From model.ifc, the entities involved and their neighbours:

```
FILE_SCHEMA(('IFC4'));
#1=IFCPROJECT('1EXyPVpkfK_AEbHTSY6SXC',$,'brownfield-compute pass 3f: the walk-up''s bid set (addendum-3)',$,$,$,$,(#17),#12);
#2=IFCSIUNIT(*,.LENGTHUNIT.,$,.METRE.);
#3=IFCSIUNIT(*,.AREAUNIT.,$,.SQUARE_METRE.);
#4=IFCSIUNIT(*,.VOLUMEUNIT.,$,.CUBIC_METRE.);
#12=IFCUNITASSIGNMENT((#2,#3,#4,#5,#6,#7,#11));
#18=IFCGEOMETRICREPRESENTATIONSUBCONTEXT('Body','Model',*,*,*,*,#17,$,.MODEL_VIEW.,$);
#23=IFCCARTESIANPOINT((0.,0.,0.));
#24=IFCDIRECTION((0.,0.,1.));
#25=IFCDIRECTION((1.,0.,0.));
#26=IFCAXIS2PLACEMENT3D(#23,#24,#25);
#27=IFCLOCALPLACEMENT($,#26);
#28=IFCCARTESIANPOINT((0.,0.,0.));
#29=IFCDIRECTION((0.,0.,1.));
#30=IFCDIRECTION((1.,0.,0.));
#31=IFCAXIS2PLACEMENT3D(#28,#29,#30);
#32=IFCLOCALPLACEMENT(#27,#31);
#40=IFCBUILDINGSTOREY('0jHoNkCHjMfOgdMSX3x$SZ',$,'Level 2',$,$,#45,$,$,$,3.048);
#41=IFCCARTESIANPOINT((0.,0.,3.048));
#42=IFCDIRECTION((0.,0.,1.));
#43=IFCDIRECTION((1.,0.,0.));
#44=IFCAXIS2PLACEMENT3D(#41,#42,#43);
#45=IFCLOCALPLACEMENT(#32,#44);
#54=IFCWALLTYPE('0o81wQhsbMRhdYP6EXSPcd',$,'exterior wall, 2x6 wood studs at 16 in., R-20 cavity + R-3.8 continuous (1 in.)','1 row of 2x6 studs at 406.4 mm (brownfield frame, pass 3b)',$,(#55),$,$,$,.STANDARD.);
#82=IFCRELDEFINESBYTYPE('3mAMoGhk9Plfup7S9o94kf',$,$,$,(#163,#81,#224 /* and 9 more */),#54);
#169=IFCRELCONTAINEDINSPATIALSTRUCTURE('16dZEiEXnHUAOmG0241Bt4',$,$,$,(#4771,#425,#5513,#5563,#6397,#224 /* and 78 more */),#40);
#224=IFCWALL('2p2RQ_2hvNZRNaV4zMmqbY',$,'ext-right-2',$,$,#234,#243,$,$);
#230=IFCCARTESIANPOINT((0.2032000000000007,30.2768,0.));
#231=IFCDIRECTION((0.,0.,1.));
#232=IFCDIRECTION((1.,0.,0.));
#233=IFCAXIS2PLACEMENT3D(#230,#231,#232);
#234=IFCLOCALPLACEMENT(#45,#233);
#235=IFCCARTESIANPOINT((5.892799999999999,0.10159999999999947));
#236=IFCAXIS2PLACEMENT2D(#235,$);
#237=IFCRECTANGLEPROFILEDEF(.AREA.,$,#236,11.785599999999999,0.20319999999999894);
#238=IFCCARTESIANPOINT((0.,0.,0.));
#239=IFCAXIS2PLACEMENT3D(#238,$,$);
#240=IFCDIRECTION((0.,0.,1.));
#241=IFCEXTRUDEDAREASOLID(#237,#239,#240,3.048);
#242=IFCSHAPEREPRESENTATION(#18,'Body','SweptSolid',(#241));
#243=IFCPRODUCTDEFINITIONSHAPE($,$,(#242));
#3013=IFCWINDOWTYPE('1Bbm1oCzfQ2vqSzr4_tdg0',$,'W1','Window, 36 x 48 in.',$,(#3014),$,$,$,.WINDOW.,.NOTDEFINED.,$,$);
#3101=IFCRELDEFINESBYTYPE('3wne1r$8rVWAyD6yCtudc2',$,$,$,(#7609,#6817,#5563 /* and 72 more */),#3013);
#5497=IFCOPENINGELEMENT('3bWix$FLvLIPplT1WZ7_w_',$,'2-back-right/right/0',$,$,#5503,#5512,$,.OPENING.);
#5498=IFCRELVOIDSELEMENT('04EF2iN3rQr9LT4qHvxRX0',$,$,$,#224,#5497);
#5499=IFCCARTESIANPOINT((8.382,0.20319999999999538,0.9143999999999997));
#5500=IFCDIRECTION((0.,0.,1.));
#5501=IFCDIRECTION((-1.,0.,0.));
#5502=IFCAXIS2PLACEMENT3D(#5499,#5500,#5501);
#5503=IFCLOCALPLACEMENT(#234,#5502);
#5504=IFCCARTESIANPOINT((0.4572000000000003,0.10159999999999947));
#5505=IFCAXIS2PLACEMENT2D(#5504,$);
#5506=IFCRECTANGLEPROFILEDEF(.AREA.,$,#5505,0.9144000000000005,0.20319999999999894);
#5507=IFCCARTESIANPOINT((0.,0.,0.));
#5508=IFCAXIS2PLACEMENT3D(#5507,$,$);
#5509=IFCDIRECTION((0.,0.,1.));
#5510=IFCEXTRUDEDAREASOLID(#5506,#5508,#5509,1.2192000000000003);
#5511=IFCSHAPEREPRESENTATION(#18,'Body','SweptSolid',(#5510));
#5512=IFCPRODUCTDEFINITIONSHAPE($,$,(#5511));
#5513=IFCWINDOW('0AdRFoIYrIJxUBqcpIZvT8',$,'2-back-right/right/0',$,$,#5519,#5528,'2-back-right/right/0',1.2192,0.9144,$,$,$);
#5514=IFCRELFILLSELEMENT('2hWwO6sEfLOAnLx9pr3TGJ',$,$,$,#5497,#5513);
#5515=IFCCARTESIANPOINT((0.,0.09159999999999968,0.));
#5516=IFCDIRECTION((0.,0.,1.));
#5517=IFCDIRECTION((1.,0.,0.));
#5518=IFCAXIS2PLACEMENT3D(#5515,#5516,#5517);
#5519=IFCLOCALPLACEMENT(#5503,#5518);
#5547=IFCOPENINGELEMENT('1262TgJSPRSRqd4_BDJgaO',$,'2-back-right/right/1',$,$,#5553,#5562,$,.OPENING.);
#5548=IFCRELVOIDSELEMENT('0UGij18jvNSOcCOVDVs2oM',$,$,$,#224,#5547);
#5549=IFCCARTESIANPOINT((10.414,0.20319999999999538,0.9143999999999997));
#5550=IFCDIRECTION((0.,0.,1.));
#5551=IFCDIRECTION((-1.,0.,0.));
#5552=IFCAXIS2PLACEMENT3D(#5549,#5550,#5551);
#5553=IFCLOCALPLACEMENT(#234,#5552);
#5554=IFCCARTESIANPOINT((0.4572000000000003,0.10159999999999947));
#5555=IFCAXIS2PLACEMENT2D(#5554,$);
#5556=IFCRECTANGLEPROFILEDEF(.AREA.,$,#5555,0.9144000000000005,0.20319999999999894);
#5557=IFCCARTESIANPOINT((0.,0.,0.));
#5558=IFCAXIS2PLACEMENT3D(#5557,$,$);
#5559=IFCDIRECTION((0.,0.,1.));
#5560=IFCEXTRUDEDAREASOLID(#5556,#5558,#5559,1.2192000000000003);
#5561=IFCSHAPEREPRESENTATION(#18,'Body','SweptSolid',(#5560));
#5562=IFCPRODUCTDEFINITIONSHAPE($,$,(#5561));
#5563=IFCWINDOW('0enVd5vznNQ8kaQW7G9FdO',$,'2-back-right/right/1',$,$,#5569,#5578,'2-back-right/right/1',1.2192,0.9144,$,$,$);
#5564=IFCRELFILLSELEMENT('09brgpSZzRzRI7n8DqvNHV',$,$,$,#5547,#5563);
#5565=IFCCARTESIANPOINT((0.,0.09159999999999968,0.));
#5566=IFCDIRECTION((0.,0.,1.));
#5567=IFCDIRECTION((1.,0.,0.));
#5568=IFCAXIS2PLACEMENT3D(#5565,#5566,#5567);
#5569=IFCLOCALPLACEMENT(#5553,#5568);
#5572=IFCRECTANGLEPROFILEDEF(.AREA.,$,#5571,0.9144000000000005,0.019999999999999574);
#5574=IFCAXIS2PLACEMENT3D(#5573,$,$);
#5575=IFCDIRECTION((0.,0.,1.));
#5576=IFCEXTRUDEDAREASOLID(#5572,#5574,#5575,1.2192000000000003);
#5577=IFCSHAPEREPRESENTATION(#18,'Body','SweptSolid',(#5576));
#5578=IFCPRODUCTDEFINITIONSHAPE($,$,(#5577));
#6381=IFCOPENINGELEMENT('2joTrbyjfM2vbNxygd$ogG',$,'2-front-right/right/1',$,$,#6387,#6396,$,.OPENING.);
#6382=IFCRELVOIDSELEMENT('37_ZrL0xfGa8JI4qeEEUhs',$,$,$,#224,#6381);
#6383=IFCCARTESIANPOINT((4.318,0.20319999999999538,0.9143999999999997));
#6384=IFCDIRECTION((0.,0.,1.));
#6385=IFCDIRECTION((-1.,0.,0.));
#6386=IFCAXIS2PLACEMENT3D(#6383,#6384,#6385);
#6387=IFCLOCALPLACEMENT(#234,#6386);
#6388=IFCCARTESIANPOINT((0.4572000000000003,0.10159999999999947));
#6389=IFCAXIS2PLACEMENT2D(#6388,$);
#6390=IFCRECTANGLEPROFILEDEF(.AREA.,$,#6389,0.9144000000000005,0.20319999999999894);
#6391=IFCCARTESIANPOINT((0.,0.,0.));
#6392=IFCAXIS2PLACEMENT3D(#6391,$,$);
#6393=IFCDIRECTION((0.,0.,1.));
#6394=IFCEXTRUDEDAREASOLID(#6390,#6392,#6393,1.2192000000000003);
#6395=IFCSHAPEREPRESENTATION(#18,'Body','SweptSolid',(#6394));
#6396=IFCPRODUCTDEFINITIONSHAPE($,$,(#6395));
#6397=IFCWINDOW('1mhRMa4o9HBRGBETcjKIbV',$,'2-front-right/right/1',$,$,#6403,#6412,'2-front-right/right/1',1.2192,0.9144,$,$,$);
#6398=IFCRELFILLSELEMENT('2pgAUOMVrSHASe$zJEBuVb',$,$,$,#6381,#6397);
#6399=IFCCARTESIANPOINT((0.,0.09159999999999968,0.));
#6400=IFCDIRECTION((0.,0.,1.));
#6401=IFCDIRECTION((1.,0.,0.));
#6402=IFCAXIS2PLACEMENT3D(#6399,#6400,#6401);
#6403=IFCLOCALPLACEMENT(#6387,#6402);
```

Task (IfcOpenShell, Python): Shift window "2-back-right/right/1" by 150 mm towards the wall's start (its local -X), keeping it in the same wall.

```python
import ifcopenshell
import ifcopenshell.api.geometry
import ifcopenshell.util.placement

model = ifcopenshell.open("model.ifc")

window = model.by_guid("0enVd5vznNQ8kaQW7G9FdO")
opening = window.FillsVoids[0].RelatingOpeningElement
wall = opening.VoidsElements[0].RelatingBuildingElement

wall_matrix = ifcopenshell.util.placement.get_local_placement(wall.ObjectPlacement)
shift = wall_matrix[:3, 0] * -0.15
before = ifcopenshell.util.placement.get_local_placement(window.ObjectPlacement)[:3, 3].copy()

# The window is placed relative to its opening, so it follows when the opening moves.
matrix = ifcopenshell.util.placement.get_local_placement(opening.ObjectPlacement)
matrix[:3, 3] += shift
ifcopenshell.api.geometry.edit_object_placement(
    model, product=opening, matrix=matrix, is_si=False, should_transform_children=True
)

after = ifcopenshell.util.placement.get_local_placement(window.ObjectPlacement)[:3, 3]
print("window moved by", (after - before).round(3) + 0.0)

model.write("model-out.ifc")
```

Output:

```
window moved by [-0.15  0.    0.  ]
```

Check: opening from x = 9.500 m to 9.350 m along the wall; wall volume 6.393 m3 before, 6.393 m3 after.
